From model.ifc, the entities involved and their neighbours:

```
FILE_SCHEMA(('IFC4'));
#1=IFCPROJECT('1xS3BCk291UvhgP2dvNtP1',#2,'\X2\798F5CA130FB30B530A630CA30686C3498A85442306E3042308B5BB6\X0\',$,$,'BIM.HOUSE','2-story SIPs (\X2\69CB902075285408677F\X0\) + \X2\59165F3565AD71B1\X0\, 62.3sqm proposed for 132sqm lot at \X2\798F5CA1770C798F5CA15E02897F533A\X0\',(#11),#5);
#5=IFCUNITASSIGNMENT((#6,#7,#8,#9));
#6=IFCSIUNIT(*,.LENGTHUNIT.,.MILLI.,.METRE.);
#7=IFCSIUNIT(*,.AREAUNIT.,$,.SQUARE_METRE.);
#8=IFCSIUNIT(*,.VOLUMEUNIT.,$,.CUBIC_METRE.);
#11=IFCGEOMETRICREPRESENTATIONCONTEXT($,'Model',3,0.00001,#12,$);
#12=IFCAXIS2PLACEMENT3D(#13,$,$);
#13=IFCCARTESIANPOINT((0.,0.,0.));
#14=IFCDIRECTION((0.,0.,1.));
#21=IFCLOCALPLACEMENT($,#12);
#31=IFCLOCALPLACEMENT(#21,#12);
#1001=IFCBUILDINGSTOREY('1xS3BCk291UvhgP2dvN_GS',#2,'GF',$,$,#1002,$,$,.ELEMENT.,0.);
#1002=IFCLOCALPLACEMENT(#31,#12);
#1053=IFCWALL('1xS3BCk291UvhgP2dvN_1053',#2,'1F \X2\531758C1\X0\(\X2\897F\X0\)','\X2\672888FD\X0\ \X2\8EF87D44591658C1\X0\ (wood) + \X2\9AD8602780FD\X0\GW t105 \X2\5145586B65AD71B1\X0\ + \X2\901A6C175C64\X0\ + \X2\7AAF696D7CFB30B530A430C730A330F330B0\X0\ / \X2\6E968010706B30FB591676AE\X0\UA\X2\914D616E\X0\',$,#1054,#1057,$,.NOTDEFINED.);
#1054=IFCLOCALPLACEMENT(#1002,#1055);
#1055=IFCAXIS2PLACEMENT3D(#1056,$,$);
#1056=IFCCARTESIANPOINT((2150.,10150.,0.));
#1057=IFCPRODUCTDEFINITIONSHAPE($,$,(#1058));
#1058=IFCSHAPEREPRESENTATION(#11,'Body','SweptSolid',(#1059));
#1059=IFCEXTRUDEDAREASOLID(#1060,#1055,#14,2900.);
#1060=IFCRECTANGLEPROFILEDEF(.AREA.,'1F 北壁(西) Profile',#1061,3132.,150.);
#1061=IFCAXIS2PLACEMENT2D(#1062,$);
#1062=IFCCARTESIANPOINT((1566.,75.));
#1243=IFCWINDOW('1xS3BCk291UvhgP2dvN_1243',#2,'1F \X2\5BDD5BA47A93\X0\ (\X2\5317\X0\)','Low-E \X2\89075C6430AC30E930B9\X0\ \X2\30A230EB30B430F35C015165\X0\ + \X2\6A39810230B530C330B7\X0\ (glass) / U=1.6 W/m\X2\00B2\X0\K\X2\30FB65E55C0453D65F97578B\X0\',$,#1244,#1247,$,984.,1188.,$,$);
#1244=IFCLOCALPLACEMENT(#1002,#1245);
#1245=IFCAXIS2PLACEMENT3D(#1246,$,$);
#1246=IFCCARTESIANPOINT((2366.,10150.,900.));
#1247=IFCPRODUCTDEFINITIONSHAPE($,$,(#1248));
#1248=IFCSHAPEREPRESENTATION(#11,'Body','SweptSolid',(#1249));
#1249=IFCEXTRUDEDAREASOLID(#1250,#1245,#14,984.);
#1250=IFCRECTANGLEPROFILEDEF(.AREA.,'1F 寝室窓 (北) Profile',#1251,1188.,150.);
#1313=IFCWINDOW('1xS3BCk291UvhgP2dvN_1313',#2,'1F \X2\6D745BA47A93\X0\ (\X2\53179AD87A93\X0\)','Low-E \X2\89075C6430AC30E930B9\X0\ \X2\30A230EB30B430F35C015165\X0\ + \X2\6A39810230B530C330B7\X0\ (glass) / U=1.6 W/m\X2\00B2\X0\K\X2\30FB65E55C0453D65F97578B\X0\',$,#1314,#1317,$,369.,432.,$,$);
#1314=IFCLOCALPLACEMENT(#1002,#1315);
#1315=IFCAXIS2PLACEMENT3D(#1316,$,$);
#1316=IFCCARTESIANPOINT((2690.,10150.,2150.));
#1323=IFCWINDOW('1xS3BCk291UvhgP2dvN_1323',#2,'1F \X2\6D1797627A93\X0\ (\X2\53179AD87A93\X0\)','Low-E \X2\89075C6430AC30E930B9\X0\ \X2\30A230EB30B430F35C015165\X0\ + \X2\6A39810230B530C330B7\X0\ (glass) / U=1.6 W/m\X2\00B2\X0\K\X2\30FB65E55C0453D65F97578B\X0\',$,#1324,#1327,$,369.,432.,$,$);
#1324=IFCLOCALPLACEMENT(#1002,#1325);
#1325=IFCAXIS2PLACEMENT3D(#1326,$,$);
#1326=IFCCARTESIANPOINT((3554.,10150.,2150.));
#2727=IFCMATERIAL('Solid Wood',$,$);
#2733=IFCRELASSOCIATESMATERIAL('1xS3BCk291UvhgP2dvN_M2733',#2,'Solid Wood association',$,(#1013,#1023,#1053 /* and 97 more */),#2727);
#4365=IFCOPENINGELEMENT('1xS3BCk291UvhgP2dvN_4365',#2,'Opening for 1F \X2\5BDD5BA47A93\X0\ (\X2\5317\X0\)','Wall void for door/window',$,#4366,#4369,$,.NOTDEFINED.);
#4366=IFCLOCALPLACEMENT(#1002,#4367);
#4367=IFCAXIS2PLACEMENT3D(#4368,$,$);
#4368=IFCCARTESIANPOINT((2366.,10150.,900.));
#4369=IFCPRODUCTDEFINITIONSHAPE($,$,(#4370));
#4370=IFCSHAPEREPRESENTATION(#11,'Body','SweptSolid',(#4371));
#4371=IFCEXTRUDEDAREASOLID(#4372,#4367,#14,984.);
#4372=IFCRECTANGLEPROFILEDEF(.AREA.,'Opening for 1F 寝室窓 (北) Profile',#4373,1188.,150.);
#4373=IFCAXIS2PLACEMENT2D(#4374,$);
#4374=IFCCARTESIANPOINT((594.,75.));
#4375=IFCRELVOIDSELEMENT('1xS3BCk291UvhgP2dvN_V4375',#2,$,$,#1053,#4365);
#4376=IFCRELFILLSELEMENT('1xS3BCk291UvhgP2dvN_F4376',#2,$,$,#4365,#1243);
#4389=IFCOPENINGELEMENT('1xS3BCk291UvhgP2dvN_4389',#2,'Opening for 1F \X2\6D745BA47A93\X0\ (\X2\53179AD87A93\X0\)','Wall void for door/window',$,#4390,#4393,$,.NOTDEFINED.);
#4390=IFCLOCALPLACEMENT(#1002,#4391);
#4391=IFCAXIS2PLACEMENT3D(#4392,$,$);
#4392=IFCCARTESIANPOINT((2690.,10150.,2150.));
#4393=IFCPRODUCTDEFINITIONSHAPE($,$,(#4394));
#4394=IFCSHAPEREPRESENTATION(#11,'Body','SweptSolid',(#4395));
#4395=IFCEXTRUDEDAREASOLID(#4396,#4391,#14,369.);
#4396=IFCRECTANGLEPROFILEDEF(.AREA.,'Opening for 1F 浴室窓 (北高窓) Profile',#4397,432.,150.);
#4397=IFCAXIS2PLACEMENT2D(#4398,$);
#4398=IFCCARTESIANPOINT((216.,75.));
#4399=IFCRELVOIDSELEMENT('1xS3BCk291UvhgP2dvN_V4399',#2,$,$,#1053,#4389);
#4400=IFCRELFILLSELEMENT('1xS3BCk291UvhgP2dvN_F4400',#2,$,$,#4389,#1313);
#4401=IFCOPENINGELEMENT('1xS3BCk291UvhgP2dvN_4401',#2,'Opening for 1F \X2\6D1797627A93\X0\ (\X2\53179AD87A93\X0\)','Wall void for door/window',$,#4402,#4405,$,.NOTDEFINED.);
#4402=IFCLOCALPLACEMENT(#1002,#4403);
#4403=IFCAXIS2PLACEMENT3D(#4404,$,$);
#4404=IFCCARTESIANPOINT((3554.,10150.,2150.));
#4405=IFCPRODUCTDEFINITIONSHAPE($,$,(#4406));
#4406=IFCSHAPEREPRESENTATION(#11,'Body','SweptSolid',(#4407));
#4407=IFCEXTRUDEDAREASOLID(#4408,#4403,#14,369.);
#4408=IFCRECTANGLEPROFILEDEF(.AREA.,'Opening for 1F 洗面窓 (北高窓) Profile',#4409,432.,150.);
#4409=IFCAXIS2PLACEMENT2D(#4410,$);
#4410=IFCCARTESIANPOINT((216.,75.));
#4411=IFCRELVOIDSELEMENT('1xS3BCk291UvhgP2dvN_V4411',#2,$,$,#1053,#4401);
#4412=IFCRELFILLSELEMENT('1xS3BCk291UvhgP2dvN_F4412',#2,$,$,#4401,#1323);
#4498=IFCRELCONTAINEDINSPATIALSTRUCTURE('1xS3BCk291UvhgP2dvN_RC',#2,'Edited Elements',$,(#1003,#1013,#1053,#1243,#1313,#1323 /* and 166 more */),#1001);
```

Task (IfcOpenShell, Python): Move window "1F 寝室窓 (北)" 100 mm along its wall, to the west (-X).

```python
import ifcopenshell
import ifcopenshell.api.geometry
import ifcopenshell.util.placement
import ifcopenshell.util.unit

model = ifcopenshell.open("model.ifc")
unit_scale = ifcopenshell.util.unit.calculate_unit_scale(model)

window = model.by_guid("1xS3BCk291UvhgP2dvN_1243")
opening = window.FillsVoids[0].RelatingOpeningElement
wall = opening.VoidsElements[0].RelatingBuildingElement

wall_matrix = ifcopenshell.util.placement.get_local_placement(wall.ObjectPlacement)
shift = wall_matrix[:3, 0] * -0.1 / unit_scale
before = ifcopenshell.util.placement.get_local_placement(window.ObjectPlacement)[:3, 3].copy()

# The window is not placed relative to its opening, so move both.
for product in (opening, window):
    matrix = ifcopenshell.util.placement.get_local_placement(product.ObjectPlacement)
    matrix[:3, 3] += shift
    ifcopenshell.api.geometry.edit_object_placement(model, product=product, matrix=matrix, is_si=False)

after = ifcopenshell.util.placement.get_local_placement(window.ObjectPlacement)[:3, 3]
print("window moved by", (after - before).round(3) + 0.0)

model.write("model-out.ifc")
```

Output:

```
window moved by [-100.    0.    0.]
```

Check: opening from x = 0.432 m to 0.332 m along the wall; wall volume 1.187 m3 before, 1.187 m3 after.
